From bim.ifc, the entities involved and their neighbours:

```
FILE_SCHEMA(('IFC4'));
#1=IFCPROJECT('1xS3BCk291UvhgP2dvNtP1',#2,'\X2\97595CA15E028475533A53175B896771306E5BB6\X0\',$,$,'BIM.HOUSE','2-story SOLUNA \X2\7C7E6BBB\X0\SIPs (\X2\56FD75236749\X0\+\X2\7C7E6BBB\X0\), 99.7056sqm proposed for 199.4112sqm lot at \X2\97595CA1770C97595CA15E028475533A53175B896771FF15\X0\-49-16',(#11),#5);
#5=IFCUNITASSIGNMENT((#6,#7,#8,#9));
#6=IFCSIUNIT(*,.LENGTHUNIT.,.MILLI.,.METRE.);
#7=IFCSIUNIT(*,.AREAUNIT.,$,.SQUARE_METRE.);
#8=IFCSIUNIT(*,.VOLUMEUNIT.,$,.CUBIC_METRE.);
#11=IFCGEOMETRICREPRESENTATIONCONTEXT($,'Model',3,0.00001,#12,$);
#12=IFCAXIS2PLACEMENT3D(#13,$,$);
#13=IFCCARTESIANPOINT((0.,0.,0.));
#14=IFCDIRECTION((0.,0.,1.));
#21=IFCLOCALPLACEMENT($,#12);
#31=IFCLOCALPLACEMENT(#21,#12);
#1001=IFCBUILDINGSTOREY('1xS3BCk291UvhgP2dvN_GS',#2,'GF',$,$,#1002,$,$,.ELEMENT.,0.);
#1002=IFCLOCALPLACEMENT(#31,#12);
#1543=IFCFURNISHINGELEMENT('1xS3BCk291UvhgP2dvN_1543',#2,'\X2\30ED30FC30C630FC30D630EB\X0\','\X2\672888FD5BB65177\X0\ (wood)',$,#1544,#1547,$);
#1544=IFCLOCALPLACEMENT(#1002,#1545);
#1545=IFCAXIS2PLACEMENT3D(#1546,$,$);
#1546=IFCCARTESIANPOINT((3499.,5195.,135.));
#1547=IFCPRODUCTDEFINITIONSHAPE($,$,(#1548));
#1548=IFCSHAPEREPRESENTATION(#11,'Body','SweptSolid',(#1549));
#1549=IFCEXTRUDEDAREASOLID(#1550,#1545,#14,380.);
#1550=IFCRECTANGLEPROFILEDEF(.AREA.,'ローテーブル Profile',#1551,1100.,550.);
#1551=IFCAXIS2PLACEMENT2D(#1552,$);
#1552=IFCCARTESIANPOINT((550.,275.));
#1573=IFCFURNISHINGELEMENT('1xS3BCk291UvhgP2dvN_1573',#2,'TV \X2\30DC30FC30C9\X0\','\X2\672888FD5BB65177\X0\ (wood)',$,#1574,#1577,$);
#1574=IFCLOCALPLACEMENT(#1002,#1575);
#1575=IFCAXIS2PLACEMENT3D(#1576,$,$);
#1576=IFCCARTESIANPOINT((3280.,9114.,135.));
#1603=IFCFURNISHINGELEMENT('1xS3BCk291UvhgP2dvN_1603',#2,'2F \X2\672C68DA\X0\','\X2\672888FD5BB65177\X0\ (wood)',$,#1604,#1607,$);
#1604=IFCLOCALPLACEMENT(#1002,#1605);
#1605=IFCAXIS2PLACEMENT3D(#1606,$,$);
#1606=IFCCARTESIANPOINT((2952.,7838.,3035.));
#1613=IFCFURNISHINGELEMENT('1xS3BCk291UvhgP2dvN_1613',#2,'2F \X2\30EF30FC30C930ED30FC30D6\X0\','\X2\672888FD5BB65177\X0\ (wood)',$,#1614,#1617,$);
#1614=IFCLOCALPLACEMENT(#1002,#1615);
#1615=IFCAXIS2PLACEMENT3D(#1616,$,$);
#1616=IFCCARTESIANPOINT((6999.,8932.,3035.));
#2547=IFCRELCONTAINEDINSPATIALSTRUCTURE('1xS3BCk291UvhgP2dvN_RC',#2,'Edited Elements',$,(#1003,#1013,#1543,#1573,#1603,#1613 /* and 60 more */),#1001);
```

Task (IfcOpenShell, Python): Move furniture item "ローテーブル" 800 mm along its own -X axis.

```python
import ifcopenshell
import ifcopenshell.api.geometry
import ifcopenshell.util.placement
import ifcopenshell.util.unit

model = ifcopenshell.open("bim.ifc")
unit_scale = ifcopenshell.util.unit.calculate_unit_scale(model)

item = model.by_guid("1xS3BCk291UvhgP2dvN_1543")
matrix = ifcopenshell.util.placement.get_local_placement(item.ObjectPlacement)
matrix[:3, 3] -= matrix[:3, 0] * 0.8 / unit_scale
ifcopenshell.api.geometry.edit_object_placement(model, product=item, matrix=matrix, is_si=False)

print(ifcopenshell.util.placement.get_local_placement(item.ObjectPlacement).round(3) + 0.0)

model.write("bim_v2.ifc")
```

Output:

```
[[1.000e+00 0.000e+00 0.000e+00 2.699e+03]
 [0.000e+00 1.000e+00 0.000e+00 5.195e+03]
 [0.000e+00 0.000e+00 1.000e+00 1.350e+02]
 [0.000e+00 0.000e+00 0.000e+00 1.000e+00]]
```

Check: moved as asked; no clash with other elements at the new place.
